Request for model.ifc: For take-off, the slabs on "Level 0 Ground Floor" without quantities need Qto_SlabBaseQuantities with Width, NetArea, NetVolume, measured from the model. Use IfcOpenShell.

First a look at what the model holds.

```python
import ifcopenshell
import ifcopenshell.util.element
import ifcopenshell.util.unit

model = ifcopenshell.open("model.ifc")
print(model.schema)
for unit_type in ("LENGTHUNIT", "AREAUNIT", "VOLUMEUNIT"):
    print(unit_type, ifcopenshell.util.unit.calculate_unit_scale(model, unit_type))
storey = next(s for s in model.by_type("IfcBuildingStorey") if s.Name == "Level 0 Ground Floor")
slabs = [e for e in ifcopenshell.util.element.get_decomposition(storey) if e.is_a("IfcSlab")]
for e in sorted(slabs, key=lambda e: e.id()):
    print(e.id(), e.is_a(), e.Name, list(ifcopenshell.util.element.get_psets(e, qtos_only=True)), sep=" | ")
```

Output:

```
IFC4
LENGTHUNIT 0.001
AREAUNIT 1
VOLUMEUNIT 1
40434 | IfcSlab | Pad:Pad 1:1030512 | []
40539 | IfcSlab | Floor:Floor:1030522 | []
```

```python
import ifcopenshell
import ifcopenshell.api.pset
import ifcopenshell.geom
import ifcopenshell.util.element
import ifcopenshell.util.shape
import ifcopenshell.util.unit

model = ifcopenshell.open("model.ifc")
unit_scale = ifcopenshell.util.unit.calculate_unit_scale(model)
area_scale = ifcopenshell.util.unit.calculate_unit_scale(model, "AREAUNIT")
volume_scale = ifcopenshell.util.unit.calculate_unit_scale(model, "VOLUMEUNIT")
settings = ifcopenshell.geom.settings()

storey = next(s for s in model.by_type("IfcBuildingStorey") if s.Name == "Level 0 Ground Floor")
slabs = [e for e in ifcopenshell.util.element.get_decomposition(storey) if e.is_a("IfcSlab")]

for e in sorted(slabs, key=lambda e: e.id()):
    if ifcopenshell.util.element.get_psets(e, qtos_only=True, should_inherit=False):
        continue
    # Geometry comes back in metres, in the element's own axes.
    shape = ifcopenshell.geom.create_shape(settings, e)
    values = {
        "Width": ifcopenshell.util.shape.get_z(shape.geometry) / unit_scale,
        "NetArea": ifcopenshell.util.shape.get_footprint_area(shape.geometry) / area_scale,
        "NetVolume": ifcopenshell.util.shape.get_volume(shape.geometry) / volume_scale,
    }
    qto = ifcopenshell.api.pset.add_qto(model, product=e, name="Qto_SlabBaseQuantities")
    ifcopenshell.api.pset.edit_qto(model, qto=qto, properties=values)
    print(e.id(), {k: round(v, 3) for k, v in values.items()})

model.write("model_v2.ifc")
```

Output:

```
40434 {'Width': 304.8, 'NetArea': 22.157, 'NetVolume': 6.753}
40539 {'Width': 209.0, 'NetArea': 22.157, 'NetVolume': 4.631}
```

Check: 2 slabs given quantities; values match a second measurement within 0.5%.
